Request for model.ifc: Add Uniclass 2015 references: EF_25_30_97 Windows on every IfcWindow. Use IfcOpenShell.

First a look at what the model holds.

```python
import ifcopenshell

model = ifcopenshell.open("model.ifc")
print(model.schema)
print("classifications:", [c.Name for c in model.by_type("IfcClassification")])
for ifc_class in ("IfcDoor", "IfcRoof", "IfcStair", "IfcWall", "IfcWindow"):
    print(ifc_class, len(model.by_type(ifc_class)))
```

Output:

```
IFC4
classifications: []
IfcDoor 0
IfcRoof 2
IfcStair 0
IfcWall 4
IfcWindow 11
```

```python
import ifcopenshell
import ifcopenshell.api.classification

model = ifcopenshell.open("model.ifc")

system = ifcopenshell.api.classification.add_classification(model, classification="Uniclass 2015")

codes = {
    "IfcWindow": ("EF_25_30_97", "Windows"),
}
for ifc_class, (code, name) in codes.items():
    products = model.by_type(ifc_class)
    ifcopenshell.api.classification.add_reference(
        model, products=products, classification=system, identification=code, name=name
    )
    print(code, len(products))

model.write("model-out.ifc")
```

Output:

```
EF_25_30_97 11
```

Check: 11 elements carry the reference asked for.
